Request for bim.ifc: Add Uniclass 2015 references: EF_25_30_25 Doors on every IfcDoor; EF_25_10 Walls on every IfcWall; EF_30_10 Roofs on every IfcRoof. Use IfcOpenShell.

First a look at what the model holds.

```python
import ifcopenshell

model = ifcopenshell.open("bim.ifc")
print(model.schema)
print("classifications:", [c.Name for c in model.by_type("IfcClassification")])
for ifc_class in ("IfcDoor", "IfcRoof", "IfcStair", "IfcWall", "IfcWindow"):
    print(ifc_class, len(model.by_type(ifc_class)))
```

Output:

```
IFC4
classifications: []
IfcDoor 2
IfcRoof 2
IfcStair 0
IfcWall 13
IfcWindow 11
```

```python
import ifcopenshell
import ifcopenshell.api.classification

model = ifcopenshell.open("bim.ifc")

system = ifcopenshell.api.classification.add_classification(model, classification="Uniclass 2015")

codes = {
    "IfcDoor": ("EF_25_30_25", "Doors"),
    "IfcWall": ("EF_25_10", "Walls"),
    "IfcRoof": ("EF_30_10", "Roofs"),
}
for ifc_class, (code, name) in codes.items():
    products = model.by_type(ifc_class)
    ifcopenshell.api.classification.add_reference(
        model, products=products, classification=system, identification=code, name=name
    )
    print(code, len(products))

model.write("bim_updated.ifc")
```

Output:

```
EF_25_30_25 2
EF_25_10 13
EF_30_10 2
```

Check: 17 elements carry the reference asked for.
